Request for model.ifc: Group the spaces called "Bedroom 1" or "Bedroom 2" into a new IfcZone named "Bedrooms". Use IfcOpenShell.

First a look at what the model holds.

```python
import ifcopenshell

model = ifcopenshell.open("model.ifc")
print(model.schema)
seen = {}
for space in model.by_type("IfcSpace"):
    seen[space.LongName] = seen.get(space.LongName, 0) + 1
for name, count in sorted(seen.items(), key=str):
    print(count, "x", name)
print("zones:", [z.Name for z in model.by_type("IfcZone")][:20])
```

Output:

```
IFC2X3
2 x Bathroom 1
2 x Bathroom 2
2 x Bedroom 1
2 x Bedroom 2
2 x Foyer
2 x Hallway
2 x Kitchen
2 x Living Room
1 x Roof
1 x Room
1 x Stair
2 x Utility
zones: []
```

```python
import ifcopenshell
import ifcopenshell.api.group
import ifcopenshell.api.root

model = ifcopenshell.open("model.ifc")

names = {"Bedroom 1", "Bedroom 2"}
spaces = [s for s in model.by_type("IfcSpace") if s.LongName in names]

zone = ifcopenshell.api.root.create_entity(model, ifc_class="IfcZone", name="Bedrooms")
ifcopenshell.api.group.assign_group(model, products=spaces, group=zone)
print(len(spaces), "spaces in", zone.Name)

model.write("model_edited.ifc")
```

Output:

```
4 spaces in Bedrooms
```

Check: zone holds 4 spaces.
